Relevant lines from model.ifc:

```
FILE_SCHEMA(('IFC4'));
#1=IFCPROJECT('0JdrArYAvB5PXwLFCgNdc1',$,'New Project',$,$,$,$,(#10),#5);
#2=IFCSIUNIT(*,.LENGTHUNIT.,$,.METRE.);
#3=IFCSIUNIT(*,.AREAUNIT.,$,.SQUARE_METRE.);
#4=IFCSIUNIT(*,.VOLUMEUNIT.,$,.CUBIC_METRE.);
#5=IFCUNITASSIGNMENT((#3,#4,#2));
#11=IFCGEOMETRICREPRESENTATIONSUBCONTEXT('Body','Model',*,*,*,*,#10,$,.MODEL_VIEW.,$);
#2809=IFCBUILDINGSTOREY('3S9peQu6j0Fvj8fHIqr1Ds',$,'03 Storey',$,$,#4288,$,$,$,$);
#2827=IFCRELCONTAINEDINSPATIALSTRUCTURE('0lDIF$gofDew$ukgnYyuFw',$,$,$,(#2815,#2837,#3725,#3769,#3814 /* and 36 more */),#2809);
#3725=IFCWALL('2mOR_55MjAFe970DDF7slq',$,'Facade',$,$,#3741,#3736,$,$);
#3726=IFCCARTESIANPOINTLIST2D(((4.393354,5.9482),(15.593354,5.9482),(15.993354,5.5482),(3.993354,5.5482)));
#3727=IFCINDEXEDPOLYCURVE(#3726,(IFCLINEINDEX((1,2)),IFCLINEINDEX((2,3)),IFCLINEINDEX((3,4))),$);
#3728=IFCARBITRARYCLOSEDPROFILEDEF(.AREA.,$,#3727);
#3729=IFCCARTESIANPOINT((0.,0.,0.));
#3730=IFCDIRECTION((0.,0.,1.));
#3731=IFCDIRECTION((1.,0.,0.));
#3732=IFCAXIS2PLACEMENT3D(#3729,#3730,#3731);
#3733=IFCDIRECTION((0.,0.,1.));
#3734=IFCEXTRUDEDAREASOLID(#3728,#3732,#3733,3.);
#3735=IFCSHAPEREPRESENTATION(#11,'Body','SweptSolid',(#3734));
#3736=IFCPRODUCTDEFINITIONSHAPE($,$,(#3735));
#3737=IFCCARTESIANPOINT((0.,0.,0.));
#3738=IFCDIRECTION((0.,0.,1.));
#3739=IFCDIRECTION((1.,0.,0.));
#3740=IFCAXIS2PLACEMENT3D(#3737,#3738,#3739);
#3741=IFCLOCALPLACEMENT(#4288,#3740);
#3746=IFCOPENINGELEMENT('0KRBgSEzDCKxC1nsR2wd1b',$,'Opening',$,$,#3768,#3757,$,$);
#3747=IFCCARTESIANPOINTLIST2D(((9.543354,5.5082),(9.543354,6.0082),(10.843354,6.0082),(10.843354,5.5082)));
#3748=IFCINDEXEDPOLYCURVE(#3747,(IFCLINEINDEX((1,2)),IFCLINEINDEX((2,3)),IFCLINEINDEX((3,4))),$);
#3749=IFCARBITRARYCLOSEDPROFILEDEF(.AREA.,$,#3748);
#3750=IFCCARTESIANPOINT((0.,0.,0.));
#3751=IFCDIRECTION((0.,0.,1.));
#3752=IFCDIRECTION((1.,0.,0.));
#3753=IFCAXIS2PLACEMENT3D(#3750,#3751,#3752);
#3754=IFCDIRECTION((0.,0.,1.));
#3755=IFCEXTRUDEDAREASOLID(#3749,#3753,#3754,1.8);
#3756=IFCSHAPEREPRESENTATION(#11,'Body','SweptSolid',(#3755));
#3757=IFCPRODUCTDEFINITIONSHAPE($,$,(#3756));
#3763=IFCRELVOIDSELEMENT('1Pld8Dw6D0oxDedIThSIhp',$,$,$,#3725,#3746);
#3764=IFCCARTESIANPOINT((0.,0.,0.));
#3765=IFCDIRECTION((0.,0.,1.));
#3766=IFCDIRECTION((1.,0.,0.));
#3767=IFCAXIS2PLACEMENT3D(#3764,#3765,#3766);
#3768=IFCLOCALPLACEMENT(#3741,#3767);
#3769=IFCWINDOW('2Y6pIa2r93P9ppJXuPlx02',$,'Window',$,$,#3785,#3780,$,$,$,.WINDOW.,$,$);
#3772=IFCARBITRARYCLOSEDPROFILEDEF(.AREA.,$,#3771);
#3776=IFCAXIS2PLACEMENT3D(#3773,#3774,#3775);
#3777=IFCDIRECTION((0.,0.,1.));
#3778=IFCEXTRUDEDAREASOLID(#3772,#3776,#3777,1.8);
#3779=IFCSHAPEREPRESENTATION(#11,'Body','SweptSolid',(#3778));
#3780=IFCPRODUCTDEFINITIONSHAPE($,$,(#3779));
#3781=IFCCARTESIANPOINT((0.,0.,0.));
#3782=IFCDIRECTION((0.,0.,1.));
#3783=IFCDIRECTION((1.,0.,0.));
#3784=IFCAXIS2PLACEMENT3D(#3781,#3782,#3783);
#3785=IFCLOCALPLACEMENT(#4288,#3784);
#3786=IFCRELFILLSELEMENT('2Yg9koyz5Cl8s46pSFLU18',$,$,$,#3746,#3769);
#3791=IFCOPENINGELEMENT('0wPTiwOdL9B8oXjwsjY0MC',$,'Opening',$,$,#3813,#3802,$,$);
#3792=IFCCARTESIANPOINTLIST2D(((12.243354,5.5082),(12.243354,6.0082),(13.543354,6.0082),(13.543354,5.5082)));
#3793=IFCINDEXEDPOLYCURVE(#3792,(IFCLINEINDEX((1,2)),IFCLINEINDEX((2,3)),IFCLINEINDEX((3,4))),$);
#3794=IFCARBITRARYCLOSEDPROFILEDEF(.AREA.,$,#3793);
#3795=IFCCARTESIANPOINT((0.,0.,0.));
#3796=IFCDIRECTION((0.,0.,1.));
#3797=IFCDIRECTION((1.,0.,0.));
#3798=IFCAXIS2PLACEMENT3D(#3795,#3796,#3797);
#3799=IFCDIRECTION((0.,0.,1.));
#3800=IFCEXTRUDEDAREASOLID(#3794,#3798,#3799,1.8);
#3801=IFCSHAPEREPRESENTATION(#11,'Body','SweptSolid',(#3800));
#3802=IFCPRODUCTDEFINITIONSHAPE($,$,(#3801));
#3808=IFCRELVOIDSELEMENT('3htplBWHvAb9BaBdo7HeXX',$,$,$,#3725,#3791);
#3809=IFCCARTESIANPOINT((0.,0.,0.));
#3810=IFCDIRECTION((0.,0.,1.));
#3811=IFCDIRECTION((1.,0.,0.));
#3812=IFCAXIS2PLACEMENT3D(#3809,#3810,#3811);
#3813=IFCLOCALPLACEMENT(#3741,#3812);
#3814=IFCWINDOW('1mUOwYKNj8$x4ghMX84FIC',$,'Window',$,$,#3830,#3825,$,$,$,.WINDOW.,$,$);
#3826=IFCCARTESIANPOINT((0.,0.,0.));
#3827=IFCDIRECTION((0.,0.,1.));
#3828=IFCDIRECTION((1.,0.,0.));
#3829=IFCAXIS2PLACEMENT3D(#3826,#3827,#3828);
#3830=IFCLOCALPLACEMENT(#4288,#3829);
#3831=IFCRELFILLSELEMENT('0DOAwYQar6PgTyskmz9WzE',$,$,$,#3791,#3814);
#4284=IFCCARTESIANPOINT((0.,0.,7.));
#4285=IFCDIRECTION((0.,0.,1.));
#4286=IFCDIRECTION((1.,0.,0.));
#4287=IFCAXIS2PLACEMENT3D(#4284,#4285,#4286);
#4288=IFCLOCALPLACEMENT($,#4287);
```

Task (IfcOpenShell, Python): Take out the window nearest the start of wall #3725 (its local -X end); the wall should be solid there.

```python
import ifcopenshell
import ifcopenshell.api.feature
import ifcopenshell.api.root
import ifcopenshell.geom
import ifcopenshell.util.shape

model = ifcopenshell.open("model.ifc")
settings = ifcopenshell.geom.settings()


def volume(element):
    """Net volume in cubic metres, openings subtracted."""
    shape = ifcopenshell.geom.create_shape(settings, element)
    return ifcopenshell.util.shape.get_volume(shape.geometry)


window = model.by_guid("2Y6pIa2r93P9ppJXuPlx02")
opening = window.FillsVoids[0].RelatingOpeningElement
wall = opening.VoidsElements[0].RelatingBuildingElement
before = volume(wall)

ifcopenshell.api.root.remove_product(model, product=window)
ifcopenshell.api.feature.remove_feature(model, feature=opening)

after = volume(wall)

print(f"wall volume {before:.3f} -> {after:.3f} m3")

model.write("model_rev.ifc")
```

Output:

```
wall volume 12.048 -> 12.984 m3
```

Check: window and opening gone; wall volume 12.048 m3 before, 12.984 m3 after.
